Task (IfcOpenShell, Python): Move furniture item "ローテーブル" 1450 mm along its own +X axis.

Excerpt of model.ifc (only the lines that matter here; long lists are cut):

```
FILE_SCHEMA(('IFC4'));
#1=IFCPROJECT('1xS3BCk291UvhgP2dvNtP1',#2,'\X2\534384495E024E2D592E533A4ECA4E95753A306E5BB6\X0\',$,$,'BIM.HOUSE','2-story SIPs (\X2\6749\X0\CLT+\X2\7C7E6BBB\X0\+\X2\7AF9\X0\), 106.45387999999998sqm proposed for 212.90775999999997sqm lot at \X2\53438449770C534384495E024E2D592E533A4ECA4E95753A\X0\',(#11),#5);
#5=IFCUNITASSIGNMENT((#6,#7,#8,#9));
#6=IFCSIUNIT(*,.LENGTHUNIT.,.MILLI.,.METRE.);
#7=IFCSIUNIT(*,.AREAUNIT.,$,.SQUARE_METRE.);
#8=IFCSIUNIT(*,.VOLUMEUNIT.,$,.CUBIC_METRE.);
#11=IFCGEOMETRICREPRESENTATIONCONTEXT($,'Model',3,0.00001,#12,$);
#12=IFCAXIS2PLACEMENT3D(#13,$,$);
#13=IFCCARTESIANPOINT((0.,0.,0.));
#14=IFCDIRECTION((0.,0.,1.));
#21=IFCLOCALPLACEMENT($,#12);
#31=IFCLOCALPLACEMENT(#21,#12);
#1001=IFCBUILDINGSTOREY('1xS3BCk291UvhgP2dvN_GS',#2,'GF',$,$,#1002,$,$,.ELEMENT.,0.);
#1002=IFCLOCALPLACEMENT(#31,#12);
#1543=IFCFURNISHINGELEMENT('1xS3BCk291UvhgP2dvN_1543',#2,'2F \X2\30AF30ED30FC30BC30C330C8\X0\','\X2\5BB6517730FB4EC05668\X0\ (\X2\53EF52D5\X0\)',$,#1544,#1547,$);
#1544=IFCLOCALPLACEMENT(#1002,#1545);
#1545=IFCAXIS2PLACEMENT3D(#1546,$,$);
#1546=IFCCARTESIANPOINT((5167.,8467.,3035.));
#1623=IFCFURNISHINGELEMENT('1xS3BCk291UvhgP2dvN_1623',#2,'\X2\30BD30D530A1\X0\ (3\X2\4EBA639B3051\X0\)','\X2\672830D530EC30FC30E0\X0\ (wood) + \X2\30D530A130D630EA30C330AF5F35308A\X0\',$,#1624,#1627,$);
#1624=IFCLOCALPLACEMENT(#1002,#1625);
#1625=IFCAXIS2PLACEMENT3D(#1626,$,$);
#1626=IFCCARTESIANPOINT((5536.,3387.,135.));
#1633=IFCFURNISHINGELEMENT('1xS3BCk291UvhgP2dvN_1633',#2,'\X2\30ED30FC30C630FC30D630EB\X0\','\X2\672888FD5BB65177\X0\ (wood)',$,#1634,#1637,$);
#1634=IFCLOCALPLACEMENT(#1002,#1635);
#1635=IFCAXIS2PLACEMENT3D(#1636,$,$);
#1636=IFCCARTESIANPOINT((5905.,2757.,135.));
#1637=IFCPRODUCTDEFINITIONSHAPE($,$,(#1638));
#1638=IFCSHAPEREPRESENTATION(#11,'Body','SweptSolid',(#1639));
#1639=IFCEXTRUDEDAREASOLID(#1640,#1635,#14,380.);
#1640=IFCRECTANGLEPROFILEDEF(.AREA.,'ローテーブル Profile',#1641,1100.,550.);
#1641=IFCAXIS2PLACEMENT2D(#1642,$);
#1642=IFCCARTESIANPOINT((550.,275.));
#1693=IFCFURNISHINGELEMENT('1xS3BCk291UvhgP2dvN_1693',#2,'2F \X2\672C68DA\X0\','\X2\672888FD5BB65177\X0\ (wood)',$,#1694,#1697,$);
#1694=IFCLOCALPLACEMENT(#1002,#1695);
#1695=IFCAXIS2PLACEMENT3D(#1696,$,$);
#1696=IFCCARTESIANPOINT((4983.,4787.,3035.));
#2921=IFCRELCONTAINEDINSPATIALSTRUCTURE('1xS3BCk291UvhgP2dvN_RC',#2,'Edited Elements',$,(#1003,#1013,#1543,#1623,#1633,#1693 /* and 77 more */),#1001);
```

```python
import ifcopenshell
import ifcopenshell.api.geometry
import ifcopenshell.util.placement
import ifcopenshell.util.unit

model = ifcopenshell.open("model.ifc")
unit_scale = ifcopenshell.util.unit.calculate_unit_scale(model)

item = model.by_guid("1xS3BCk291UvhgP2dvN_1633")
matrix = ifcopenshell.util.placement.get_local_placement(item.ObjectPlacement)
matrix[:3, 3] += matrix[:3, 0] * 1.45 / unit_scale
ifcopenshell.api.geometry.edit_object_placement(model, product=item, matrix=matrix, is_si=False)

print(ifcopenshell.util.placement.get_local_placement(item.ObjectPlacement).round(3) + 0.0)

model.write("model_updated.ifc")
```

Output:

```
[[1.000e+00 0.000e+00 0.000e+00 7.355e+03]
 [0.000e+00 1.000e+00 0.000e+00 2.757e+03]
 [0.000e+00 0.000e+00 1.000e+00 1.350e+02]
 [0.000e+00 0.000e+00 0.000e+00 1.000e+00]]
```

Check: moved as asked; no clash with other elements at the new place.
